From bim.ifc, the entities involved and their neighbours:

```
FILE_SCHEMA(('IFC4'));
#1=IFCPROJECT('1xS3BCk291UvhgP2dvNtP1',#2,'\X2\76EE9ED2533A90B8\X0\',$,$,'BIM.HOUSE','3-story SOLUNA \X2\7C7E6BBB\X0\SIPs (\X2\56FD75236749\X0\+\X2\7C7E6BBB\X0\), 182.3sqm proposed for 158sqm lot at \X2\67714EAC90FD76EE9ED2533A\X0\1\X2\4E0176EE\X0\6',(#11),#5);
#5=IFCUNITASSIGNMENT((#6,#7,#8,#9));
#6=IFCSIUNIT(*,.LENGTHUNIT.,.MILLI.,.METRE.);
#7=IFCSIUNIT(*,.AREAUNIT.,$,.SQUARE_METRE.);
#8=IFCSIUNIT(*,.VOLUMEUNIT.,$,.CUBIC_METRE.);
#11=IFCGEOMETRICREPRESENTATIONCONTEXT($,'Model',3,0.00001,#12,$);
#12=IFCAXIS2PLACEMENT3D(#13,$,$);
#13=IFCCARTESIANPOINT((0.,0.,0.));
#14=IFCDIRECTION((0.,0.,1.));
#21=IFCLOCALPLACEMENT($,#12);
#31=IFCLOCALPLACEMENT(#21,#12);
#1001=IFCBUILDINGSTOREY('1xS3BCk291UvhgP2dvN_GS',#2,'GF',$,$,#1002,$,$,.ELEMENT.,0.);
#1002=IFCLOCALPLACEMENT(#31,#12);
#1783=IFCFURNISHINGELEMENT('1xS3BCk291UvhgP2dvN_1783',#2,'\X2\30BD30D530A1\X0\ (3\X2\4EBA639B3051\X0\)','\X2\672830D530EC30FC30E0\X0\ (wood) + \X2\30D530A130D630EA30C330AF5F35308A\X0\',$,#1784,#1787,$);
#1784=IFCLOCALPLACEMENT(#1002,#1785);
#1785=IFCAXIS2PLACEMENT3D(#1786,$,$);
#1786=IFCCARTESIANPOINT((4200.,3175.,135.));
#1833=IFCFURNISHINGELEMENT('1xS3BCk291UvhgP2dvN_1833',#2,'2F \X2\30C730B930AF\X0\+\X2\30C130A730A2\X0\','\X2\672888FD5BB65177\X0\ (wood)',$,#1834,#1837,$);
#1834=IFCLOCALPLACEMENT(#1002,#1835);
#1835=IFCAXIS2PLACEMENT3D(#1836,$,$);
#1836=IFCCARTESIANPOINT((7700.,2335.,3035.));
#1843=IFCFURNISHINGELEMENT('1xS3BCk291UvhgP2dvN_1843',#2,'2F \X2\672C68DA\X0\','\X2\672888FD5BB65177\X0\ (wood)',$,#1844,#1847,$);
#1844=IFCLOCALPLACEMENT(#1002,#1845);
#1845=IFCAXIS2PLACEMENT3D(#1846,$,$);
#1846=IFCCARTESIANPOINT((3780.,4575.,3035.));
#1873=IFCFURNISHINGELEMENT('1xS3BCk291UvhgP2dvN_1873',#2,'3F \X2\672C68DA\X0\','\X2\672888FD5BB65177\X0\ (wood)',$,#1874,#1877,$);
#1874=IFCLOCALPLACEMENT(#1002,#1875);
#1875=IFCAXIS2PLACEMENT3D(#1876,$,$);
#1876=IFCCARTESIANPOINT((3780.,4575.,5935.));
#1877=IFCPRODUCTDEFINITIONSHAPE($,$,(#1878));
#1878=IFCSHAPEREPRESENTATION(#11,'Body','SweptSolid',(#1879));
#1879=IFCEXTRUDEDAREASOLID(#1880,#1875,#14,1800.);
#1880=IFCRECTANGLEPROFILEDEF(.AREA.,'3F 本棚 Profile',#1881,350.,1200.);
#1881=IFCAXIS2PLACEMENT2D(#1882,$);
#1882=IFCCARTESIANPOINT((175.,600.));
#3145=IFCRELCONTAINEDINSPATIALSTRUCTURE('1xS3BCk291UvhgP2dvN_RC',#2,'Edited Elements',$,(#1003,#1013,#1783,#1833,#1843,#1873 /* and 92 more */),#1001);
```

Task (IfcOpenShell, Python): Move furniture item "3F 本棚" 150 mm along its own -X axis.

```python
import ifcopenshell
import ifcopenshell.api.geometry
import ifcopenshell.util.placement
import ifcopenshell.util.unit

model = ifcopenshell.open("bim.ifc")
unit_scale = ifcopenshell.util.unit.calculate_unit_scale(model)

item = model.by_guid("1xS3BCk291UvhgP2dvN_1873")
matrix = ifcopenshell.util.placement.get_local_placement(item.ObjectPlacement)
matrix[:3, 3] -= matrix[:3, 0] * 0.15 / unit_scale
ifcopenshell.api.geometry.edit_object_placement(model, product=item, matrix=matrix, is_si=False)

print(ifcopenshell.util.placement.get_local_placement(item.ObjectPlacement).round(3) + 0.0)

model.write("bim_rev.ifc")
```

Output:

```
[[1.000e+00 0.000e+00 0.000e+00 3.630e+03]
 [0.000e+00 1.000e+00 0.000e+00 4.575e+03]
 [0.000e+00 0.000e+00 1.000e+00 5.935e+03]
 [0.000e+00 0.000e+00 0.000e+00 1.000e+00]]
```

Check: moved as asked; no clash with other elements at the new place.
